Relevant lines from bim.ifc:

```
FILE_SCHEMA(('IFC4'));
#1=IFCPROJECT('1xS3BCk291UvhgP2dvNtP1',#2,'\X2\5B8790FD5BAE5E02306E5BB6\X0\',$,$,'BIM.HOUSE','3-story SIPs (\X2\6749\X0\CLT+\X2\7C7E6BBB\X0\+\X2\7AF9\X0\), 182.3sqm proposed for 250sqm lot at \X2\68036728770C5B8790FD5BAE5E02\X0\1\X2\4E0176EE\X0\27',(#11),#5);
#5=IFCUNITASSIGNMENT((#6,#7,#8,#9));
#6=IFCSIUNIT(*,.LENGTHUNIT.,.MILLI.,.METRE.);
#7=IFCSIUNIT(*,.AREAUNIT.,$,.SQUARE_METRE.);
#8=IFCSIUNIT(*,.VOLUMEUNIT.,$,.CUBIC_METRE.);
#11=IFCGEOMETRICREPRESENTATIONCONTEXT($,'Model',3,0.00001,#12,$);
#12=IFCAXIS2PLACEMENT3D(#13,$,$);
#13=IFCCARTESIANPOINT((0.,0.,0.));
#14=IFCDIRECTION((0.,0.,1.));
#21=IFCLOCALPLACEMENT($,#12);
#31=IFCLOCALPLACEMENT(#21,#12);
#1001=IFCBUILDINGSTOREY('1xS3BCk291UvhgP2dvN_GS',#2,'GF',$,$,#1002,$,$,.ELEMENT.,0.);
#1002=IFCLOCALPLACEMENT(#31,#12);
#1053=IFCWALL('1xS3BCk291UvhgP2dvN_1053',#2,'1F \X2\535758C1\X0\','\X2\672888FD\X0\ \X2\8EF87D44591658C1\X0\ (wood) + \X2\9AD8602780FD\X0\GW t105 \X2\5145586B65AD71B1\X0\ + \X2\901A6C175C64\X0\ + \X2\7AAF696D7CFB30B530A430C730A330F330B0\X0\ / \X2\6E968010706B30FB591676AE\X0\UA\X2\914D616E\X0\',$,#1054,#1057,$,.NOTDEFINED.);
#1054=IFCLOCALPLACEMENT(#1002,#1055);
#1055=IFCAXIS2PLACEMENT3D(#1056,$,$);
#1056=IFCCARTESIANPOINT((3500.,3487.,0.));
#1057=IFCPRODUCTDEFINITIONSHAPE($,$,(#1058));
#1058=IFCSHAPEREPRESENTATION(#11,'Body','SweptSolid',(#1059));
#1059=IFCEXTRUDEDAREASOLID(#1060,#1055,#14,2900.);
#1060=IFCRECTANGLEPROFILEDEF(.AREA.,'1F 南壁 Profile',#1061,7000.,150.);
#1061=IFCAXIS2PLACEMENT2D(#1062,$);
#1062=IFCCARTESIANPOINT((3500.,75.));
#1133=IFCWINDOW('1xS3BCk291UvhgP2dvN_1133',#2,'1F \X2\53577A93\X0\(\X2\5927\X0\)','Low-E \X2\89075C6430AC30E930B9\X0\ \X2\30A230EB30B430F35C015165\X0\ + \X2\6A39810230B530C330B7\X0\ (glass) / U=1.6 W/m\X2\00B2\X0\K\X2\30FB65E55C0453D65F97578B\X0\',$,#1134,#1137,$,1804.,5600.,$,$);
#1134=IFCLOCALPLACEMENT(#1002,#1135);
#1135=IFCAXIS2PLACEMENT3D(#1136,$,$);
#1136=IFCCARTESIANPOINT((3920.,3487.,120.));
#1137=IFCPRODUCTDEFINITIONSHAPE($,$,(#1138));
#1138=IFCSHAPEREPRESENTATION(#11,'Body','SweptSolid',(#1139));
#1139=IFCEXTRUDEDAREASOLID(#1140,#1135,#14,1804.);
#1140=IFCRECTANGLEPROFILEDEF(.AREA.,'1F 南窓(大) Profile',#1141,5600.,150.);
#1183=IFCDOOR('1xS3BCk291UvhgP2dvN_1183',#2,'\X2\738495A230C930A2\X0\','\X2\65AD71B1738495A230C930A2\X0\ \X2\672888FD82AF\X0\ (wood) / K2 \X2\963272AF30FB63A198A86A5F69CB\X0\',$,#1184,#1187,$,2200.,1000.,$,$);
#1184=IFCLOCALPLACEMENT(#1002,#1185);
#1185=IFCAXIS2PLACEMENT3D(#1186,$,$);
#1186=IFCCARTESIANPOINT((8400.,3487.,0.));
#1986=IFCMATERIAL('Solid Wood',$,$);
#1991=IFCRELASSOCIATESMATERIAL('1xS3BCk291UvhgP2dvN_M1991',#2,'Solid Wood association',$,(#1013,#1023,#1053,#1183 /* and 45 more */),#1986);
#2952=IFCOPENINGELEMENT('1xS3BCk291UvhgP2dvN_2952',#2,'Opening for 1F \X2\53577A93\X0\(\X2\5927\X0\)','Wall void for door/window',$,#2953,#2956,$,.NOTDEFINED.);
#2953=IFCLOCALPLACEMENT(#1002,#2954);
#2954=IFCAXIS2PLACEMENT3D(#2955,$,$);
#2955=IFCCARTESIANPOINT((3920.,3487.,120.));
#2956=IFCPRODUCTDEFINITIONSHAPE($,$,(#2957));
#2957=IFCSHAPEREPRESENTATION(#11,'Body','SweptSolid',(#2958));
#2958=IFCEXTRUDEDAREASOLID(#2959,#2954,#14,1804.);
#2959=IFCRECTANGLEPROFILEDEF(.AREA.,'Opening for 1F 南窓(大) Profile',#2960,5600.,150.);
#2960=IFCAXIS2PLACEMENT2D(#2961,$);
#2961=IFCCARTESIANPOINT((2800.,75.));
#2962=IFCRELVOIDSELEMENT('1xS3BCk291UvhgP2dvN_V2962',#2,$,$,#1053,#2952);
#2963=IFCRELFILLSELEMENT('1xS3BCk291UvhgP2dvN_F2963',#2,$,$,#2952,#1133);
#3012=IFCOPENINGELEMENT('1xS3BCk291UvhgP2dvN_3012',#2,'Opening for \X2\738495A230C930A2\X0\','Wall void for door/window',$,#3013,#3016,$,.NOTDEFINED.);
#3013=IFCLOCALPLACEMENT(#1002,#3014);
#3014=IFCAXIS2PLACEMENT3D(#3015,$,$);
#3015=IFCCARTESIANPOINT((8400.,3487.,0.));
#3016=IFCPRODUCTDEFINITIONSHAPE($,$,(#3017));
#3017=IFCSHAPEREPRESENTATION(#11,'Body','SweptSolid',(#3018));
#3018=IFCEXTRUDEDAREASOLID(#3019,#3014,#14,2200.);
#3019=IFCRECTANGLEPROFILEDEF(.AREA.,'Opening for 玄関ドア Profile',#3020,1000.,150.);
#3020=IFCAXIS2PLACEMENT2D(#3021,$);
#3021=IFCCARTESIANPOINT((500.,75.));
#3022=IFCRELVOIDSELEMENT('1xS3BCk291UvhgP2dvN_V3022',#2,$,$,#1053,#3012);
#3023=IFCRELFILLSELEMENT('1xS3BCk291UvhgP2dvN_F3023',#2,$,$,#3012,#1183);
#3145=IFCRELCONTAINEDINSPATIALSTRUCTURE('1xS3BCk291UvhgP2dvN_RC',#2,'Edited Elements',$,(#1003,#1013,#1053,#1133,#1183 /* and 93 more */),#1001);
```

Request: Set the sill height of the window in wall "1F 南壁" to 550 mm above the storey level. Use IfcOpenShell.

```python
import numpy as np
import ifcopenshell
import ifcopenshell.api.geometry
import ifcopenshell.geom
import ifcopenshell.util.element
import ifcopenshell.util.placement
import ifcopenshell.util.shape
import ifcopenshell.util.unit

model = ifcopenshell.open("bim.ifc")
unit_scale = ifcopenshell.util.unit.calculate_unit_scale(model)

window = model.by_guid("1xS3BCk291UvhgP2dvN_1133")
opening = window.FillsVoids[0].RelatingOpeningElement
storey = ifcopenshell.util.element.get_container(window, ifc_class="IfcBuildingStorey")
level = ifcopenshell.util.placement.get_local_placement(storey.ObjectPlacement)[2, 3]

# The opening's origin need not be at the sill, so measure its lowest point.
shape = ifcopenshell.geom.create_shape(ifcopenshell.geom.settings(), opening)
bottom = ifcopenshell.util.shape.get_shape_bottom_elevation(shape, shape.geometry) / unit_scale
dz = level + 550.0 - bottom

shift = np.array([0.0, 0.0, dz])
# The window is not placed relative to its opening, so move both.
for product in (opening, window):
    matrix = ifcopenshell.util.placement.get_local_placement(product.ObjectPlacement)
    matrix[:3, 3] += shift
    ifcopenshell.api.geometry.edit_object_placement(model, product=product, matrix=matrix, is_si=False)

print(f"moved by {dz * unit_scale:+.3f} m")

model.write("bim-out.ifc")
```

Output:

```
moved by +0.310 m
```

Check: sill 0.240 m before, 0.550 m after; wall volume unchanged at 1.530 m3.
